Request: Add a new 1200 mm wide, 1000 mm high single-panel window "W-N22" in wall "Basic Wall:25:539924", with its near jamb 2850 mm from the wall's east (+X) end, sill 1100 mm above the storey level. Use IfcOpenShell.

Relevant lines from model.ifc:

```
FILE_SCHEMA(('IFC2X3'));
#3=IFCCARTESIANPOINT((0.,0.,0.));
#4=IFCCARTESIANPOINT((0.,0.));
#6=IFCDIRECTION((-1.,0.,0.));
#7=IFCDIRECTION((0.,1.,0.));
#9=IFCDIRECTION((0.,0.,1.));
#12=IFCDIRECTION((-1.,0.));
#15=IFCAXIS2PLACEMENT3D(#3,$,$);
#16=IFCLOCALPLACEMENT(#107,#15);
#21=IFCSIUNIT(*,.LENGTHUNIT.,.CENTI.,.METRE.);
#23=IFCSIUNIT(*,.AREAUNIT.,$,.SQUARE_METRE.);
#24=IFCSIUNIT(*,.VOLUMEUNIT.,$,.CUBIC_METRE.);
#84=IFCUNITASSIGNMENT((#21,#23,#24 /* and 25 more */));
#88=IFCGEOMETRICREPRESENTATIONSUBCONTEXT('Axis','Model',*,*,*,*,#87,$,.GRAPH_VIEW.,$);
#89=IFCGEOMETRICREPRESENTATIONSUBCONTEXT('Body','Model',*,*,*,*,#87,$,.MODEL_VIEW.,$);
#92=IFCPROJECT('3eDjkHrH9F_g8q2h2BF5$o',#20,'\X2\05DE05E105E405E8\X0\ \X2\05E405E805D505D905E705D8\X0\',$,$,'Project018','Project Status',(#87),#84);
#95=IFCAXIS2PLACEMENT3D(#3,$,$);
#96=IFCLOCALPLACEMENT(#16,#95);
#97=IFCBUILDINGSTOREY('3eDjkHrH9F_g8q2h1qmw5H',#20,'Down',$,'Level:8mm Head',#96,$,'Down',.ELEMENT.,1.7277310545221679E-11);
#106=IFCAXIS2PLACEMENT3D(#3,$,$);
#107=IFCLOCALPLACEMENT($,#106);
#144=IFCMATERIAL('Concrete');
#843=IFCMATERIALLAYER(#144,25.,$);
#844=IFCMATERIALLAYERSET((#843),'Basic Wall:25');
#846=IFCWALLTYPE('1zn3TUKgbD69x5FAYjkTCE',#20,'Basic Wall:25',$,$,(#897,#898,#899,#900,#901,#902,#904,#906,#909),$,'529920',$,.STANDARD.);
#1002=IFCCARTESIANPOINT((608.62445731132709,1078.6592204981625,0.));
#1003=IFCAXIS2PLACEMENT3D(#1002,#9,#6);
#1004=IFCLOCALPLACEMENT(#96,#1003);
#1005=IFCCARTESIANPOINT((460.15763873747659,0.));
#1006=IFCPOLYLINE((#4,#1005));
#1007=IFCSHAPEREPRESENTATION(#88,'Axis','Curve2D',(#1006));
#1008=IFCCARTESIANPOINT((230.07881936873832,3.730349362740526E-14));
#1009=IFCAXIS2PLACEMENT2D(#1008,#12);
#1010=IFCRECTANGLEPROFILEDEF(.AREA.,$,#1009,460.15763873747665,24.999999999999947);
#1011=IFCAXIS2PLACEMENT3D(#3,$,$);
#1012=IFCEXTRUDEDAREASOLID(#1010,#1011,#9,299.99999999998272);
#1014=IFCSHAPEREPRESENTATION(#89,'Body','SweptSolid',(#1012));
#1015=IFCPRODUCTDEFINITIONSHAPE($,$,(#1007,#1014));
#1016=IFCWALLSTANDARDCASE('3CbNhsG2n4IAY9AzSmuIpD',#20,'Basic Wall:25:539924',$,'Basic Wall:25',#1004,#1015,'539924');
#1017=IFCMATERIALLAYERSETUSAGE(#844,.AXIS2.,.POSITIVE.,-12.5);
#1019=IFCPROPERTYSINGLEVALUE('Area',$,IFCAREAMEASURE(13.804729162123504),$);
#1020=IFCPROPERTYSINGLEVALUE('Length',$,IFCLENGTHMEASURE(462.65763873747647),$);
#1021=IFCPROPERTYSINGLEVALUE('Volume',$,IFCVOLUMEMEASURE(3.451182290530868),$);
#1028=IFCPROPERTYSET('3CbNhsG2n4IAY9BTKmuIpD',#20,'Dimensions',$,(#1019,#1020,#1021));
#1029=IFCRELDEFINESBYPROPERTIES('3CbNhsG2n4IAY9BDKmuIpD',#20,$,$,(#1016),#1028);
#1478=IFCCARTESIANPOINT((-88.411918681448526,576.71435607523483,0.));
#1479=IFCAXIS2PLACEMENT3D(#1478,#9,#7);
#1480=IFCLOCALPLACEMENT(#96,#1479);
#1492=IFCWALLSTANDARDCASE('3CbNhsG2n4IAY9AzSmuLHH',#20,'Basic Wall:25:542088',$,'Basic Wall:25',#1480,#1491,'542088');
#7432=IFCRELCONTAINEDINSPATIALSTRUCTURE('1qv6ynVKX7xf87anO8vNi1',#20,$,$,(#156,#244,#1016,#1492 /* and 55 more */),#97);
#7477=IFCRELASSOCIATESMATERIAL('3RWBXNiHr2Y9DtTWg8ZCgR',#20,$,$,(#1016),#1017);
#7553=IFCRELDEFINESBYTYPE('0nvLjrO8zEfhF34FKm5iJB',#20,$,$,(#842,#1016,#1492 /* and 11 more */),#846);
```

```python
import numpy as np
import ifcopenshell
import ifcopenshell.api.feature
import ifcopenshell.api.geometry
import ifcopenshell.api.pset
import ifcopenshell.api.root
import ifcopenshell.api.spatial
import ifcopenshell.api.type
import ifcopenshell.geom
import ifcopenshell.util.element
import ifcopenshell.util.placement
import ifcopenshell.util.representation
import ifcopenshell.util.shape
import ifcopenshell.util.unit

model = ifcopenshell.open("model.ifc")
unit_scale = ifcopenshell.util.unit.calculate_unit_scale(model)
area_scale = ifcopenshell.util.unit.calculate_unit_scale(model, "AREAUNIT")
volume_scale = ifcopenshell.util.unit.calculate_unit_scale(model, "VOLUMEUNIT")
settings = ifcopenshell.geom.settings()


def volume(element):
    """Net volume in cubic metres, openings subtracted."""
    shape = ifcopenshell.geom.create_shape(settings, element)
    return ifcopenshell.util.shape.get_volume(shape.geometry)


wall = model.by_id(1016)
storey = ifcopenshell.util.element.get_container(wall, ifc_class="IfcBuildingStorey")
context = ifcopenshell.util.representation.get_context(model, "Model", "Body", "MODEL_VIEW")
before = volume(wall)

width, height, from_end, sill = 1.2, 1, 2.85, 1.1  # metres

# The wall runs along its own X axis, and the end named is its -X end.
wall_shape = ifcopenshell.geom.create_shape(settings, wall)
x, y, z = ifcopenshell.util.shape.get_vertices(wall_shape.geometry).T
start = x.min() + from_end
face, thickness = float(y.min()), float(y.max() - y.min())
wall_matrix = ifcopenshell.util.placement.get_local_placement(wall.ObjectPlacement)
level = ifcopenshell.util.placement.get_local_placement(storey.ObjectPlacement)[2, 3]


def in_wall(x, y):
    """Placement at x, y metres in the wall's axes, at sill height."""
    matrix = wall_matrix.copy()
    matrix[:, 3] = wall_matrix @ np.array([x / unit_scale, y / unit_scale, 0.0, 1.0])
    matrix[2, 3] = level + sill / unit_scale
    return matrix


# Opening: a box that overshoots both wall faces by 50 mm.
opening = ifcopenshell.api.root.create_entity(model, ifc_class="IfcOpeningElement")
box = ifcopenshell.api.geometry.add_wall_representation(
    model, context=context, length=width, height=height, thickness=thickness + 0.1
)
ifcopenshell.api.geometry.assign_representation(model, product=opening, representation=box)
ifcopenshell.api.geometry.edit_object_placement(model, product=opening, matrix=in_wall(start, face - 0.05), is_si=False)
ifcopenshell.api.feature.add_feature(model, feature=opening, element=wall)

window = ifcopenshell.api.root.create_entity(model, ifc_class="IfcWindow", name="W-N22")
window.OverallWidth, window.OverallHeight = width / unit_scale, height / unit_scale
body = ifcopenshell.api.geometry.add_window_representation(
    model,
    context=context,
    overall_width=window.OverallWidth,
    overall_height=window.OverallHeight,
    partition_type="SINGLE_PANEL",
)
ifcopenshell.api.geometry.assign_representation(model, product=window, representation=body)
ifcopenshell.api.spatial.assign_container(model, products=[window], relating_structure=storey)
fills = ifcopenshell.api.feature.add_filling(model, opening=opening, element=window)
fills.OwnerHistory = window.OwnerHistory  # required in IFC2X3

# IFC2X3 keeps the operation on the window style.
style = ifcopenshell.api.root.create_entity(model, ifc_class="IfcWindowStyle", name="W-N22")
style.OperationType, style.ConstructionType = "SINGLE_PANEL", "NOTDEFINED"
style.ParameterTakesPrecedence = style.Sizeable = False
ifcopenshell.api.type.assign_type(model, related_objects=[window], relating_type=style)

# Centre the window in the wall's thickness.
ifcopenshell.api.geometry.edit_object_placement(model, product=window, matrix=in_wall(start, face), is_si=False)
window_shape = ifcopenshell.geom.create_shape(settings, window)
depth = ifcopenshell.util.shape.get_vertices(window_shape.geometry)[:, 1]
offset = face + thickness / 2 - (depth.min() + depth.max()) / 2
ifcopenshell.api.geometry.edit_object_placement(model, product=window, matrix=in_wall(start, offset), is_si=False)

after = volume(wall)

# Update the wall's stored quantities.
pset = model.by_id(ifcopenshell.util.element.get_pset(wall, "Dimensions", should_inherit=False)["id"])
ifcopenshell.api.pset.edit_pset(model, pset=pset, properties={
    "Area": model.create_entity("IfcAreaMeasure", after / thickness / area_scale),
    "Volume": model.create_entity("IfcVolumeMeasure", after / volume_scale),
})

print(f"wall volume {before:.3f} -> {after:.3f} m3")

model.write("model_v2.ifc")
```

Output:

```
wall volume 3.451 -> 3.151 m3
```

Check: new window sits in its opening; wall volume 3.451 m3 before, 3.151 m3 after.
